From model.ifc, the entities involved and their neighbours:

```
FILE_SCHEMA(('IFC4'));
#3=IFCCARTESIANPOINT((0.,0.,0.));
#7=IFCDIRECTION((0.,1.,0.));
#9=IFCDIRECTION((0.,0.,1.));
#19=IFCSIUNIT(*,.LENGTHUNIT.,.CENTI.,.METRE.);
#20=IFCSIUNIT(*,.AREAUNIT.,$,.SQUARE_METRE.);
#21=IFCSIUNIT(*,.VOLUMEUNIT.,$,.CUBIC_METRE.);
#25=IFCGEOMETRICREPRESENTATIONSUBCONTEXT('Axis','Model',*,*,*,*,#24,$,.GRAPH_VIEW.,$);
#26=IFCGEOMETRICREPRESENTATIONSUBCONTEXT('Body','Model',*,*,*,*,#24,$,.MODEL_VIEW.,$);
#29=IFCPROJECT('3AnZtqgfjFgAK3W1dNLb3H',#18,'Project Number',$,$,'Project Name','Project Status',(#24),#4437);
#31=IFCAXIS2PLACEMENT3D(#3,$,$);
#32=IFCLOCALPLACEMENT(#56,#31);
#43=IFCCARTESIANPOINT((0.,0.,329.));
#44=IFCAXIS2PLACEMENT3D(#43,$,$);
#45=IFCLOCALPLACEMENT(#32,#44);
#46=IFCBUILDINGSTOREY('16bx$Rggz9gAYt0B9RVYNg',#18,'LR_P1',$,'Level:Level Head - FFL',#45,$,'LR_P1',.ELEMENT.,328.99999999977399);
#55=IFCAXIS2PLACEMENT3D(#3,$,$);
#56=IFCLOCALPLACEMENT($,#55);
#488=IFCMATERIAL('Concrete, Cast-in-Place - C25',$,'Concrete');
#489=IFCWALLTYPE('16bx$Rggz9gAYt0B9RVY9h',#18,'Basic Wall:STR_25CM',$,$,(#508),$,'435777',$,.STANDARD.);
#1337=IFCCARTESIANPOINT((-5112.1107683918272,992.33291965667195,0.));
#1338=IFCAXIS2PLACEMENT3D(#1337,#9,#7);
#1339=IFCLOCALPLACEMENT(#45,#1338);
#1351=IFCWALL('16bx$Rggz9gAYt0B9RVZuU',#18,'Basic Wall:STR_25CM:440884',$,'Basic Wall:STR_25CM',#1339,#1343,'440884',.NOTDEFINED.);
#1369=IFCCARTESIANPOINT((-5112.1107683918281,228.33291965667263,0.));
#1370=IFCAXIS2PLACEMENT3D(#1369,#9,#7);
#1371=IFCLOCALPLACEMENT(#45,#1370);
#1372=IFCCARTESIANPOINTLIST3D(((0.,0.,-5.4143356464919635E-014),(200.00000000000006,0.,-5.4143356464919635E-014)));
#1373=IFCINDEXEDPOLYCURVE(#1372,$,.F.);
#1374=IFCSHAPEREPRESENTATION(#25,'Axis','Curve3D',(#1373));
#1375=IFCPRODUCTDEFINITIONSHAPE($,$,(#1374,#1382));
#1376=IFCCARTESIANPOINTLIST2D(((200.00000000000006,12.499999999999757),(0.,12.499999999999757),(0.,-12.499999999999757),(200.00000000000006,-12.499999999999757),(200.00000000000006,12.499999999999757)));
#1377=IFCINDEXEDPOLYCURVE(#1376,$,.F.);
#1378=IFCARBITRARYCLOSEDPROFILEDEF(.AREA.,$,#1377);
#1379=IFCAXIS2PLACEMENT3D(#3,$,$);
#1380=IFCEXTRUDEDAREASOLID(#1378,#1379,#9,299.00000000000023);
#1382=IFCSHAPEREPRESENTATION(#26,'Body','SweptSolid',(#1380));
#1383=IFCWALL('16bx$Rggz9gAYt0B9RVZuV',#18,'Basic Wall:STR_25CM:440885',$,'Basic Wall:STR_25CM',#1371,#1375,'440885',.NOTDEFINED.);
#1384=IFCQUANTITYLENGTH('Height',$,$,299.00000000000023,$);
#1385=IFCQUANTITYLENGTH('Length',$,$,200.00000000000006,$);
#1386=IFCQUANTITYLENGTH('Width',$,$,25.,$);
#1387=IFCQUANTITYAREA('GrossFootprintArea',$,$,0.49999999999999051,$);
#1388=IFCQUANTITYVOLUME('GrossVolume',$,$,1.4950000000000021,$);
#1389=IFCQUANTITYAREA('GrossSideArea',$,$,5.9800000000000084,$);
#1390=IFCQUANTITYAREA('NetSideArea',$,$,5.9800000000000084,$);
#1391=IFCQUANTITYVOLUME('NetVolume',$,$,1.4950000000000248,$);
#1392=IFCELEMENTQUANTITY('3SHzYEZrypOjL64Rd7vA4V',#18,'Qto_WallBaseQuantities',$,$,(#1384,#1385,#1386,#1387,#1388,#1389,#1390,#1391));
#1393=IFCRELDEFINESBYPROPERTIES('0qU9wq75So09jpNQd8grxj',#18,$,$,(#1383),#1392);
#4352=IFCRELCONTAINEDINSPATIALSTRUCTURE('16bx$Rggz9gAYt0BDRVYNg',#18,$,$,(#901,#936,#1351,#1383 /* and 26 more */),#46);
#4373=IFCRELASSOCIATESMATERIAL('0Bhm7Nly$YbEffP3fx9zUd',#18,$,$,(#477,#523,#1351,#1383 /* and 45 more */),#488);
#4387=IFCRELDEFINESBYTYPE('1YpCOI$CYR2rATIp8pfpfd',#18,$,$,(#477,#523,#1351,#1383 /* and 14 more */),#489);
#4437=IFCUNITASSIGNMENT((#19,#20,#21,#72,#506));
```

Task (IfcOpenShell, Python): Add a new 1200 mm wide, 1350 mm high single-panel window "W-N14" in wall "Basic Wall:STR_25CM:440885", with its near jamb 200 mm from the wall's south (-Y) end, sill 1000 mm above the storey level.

```python
import numpy as np
import ifcopenshell
import ifcopenshell.api.feature
import ifcopenshell.api.geometry
import ifcopenshell.api.pset
import ifcopenshell.api.root
import ifcopenshell.api.spatial
import ifcopenshell.geom
import ifcopenshell.util.element
import ifcopenshell.util.placement
import ifcopenshell.util.representation
import ifcopenshell.util.shape
import ifcopenshell.util.unit

model = ifcopenshell.open("model.ifc")
unit_scale = ifcopenshell.util.unit.calculate_unit_scale(model)
area_scale = ifcopenshell.util.unit.calculate_unit_scale(model, "AREAUNIT")
volume_scale = ifcopenshell.util.unit.calculate_unit_scale(model, "VOLUMEUNIT")
settings = ifcopenshell.geom.settings()


def volume(element):
    """Net volume in cubic metres, openings subtracted."""
    shape = ifcopenshell.geom.create_shape(settings, element)
    return ifcopenshell.util.shape.get_volume(shape.geometry)


wall = model.by_guid("16bx$Rggz9gAYt0B9RVZuV")
storey = ifcopenshell.util.element.get_container(wall, ifc_class="IfcBuildingStorey")
context = ifcopenshell.util.representation.get_context(model, "Model", "Body", "MODEL_VIEW")
before = volume(wall)

width, height, from_end, sill = 1.2, 1.35, 0.2, 1  # metres

# The wall runs along its own X axis, and the end named is its -X end.
wall_shape = ifcopenshell.geom.create_shape(settings, wall)
x, y, z = ifcopenshell.util.shape.get_vertices(wall_shape.geometry).T
start = x.min() + from_end
face, thickness = float(y.min()), float(y.max() - y.min())
wall_matrix = ifcopenshell.util.placement.get_local_placement(wall.ObjectPlacement)
level = ifcopenshell.util.placement.get_local_placement(storey.ObjectPlacement)[2, 3]


def in_wall(x, y):
    """Placement at x, y metres in the wall's axes, at sill height."""
    matrix = wall_matrix.copy()
    matrix[:, 3] = wall_matrix @ np.array([x / unit_scale, y / unit_scale, 0.0, 1.0])
    matrix[2, 3] = level + sill / unit_scale
    return matrix


# Opening: a box that overshoots both wall faces by 50 mm.
opening = ifcopenshell.api.root.create_entity(model, ifc_class="IfcOpeningElement", predefined_type="OPENING")
box = ifcopenshell.api.geometry.add_wall_representation(
    model, context=context, length=width, height=height, thickness=thickness + 0.1
)
ifcopenshell.api.geometry.assign_representation(model, product=opening, representation=box)
ifcopenshell.api.geometry.edit_object_placement(model, product=opening, matrix=in_wall(start, face - 0.05), is_si=False)
ifcopenshell.api.feature.add_feature(model, feature=opening, element=wall)

window = ifcopenshell.api.root.create_entity(model, ifc_class="IfcWindow", name="W-N14", predefined_type="WINDOW")
window.OverallWidth, window.OverallHeight = width / unit_scale, height / unit_scale
window.PartitioningType = "SINGLE_PANEL"
body = ifcopenshell.api.geometry.add_window_representation(
    model,
    context=context,
    overall_width=window.OverallWidth,
    overall_height=window.OverallHeight,
    partition_type="SINGLE_PANEL",
)
ifcopenshell.api.geometry.assign_representation(model, product=window, representation=body)
ifcopenshell.api.spatial.assign_container(model, products=[window], relating_structure=storey)
ifcopenshell.api.feature.add_filling(model, opening=opening, element=window)

# Centre the window in the wall's thickness.
ifcopenshell.api.geometry.edit_object_placement(model, product=window, matrix=in_wall(start, face), is_si=False)
window_shape = ifcopenshell.geom.create_shape(settings, window)
depth = ifcopenshell.util.shape.get_vertices(window_shape.geometry)[:, 1]
offset = face + thickness / 2 - (depth.min() + depth.max()) / 2
ifcopenshell.api.geometry.edit_object_placement(model, product=window, matrix=in_wall(start, offset), is_si=False)

after = volume(wall)

# Update the wall's stored quantities.
qto = model.by_id(ifcopenshell.util.element.get_pset(wall, "Qto_WallBaseQuantities", should_inherit=False)["id"])
ifcopenshell.api.pset.edit_qto(model, qto=qto, properties={
    "NetSideArea": after / thickness / area_scale,
    "NetVolume": after / volume_scale,
})

print(f"wall volume {before:.3f} -> {after:.3f} m3")

model.write("model_rev.ifc")
```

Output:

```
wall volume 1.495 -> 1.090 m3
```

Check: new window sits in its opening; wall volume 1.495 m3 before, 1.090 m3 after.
